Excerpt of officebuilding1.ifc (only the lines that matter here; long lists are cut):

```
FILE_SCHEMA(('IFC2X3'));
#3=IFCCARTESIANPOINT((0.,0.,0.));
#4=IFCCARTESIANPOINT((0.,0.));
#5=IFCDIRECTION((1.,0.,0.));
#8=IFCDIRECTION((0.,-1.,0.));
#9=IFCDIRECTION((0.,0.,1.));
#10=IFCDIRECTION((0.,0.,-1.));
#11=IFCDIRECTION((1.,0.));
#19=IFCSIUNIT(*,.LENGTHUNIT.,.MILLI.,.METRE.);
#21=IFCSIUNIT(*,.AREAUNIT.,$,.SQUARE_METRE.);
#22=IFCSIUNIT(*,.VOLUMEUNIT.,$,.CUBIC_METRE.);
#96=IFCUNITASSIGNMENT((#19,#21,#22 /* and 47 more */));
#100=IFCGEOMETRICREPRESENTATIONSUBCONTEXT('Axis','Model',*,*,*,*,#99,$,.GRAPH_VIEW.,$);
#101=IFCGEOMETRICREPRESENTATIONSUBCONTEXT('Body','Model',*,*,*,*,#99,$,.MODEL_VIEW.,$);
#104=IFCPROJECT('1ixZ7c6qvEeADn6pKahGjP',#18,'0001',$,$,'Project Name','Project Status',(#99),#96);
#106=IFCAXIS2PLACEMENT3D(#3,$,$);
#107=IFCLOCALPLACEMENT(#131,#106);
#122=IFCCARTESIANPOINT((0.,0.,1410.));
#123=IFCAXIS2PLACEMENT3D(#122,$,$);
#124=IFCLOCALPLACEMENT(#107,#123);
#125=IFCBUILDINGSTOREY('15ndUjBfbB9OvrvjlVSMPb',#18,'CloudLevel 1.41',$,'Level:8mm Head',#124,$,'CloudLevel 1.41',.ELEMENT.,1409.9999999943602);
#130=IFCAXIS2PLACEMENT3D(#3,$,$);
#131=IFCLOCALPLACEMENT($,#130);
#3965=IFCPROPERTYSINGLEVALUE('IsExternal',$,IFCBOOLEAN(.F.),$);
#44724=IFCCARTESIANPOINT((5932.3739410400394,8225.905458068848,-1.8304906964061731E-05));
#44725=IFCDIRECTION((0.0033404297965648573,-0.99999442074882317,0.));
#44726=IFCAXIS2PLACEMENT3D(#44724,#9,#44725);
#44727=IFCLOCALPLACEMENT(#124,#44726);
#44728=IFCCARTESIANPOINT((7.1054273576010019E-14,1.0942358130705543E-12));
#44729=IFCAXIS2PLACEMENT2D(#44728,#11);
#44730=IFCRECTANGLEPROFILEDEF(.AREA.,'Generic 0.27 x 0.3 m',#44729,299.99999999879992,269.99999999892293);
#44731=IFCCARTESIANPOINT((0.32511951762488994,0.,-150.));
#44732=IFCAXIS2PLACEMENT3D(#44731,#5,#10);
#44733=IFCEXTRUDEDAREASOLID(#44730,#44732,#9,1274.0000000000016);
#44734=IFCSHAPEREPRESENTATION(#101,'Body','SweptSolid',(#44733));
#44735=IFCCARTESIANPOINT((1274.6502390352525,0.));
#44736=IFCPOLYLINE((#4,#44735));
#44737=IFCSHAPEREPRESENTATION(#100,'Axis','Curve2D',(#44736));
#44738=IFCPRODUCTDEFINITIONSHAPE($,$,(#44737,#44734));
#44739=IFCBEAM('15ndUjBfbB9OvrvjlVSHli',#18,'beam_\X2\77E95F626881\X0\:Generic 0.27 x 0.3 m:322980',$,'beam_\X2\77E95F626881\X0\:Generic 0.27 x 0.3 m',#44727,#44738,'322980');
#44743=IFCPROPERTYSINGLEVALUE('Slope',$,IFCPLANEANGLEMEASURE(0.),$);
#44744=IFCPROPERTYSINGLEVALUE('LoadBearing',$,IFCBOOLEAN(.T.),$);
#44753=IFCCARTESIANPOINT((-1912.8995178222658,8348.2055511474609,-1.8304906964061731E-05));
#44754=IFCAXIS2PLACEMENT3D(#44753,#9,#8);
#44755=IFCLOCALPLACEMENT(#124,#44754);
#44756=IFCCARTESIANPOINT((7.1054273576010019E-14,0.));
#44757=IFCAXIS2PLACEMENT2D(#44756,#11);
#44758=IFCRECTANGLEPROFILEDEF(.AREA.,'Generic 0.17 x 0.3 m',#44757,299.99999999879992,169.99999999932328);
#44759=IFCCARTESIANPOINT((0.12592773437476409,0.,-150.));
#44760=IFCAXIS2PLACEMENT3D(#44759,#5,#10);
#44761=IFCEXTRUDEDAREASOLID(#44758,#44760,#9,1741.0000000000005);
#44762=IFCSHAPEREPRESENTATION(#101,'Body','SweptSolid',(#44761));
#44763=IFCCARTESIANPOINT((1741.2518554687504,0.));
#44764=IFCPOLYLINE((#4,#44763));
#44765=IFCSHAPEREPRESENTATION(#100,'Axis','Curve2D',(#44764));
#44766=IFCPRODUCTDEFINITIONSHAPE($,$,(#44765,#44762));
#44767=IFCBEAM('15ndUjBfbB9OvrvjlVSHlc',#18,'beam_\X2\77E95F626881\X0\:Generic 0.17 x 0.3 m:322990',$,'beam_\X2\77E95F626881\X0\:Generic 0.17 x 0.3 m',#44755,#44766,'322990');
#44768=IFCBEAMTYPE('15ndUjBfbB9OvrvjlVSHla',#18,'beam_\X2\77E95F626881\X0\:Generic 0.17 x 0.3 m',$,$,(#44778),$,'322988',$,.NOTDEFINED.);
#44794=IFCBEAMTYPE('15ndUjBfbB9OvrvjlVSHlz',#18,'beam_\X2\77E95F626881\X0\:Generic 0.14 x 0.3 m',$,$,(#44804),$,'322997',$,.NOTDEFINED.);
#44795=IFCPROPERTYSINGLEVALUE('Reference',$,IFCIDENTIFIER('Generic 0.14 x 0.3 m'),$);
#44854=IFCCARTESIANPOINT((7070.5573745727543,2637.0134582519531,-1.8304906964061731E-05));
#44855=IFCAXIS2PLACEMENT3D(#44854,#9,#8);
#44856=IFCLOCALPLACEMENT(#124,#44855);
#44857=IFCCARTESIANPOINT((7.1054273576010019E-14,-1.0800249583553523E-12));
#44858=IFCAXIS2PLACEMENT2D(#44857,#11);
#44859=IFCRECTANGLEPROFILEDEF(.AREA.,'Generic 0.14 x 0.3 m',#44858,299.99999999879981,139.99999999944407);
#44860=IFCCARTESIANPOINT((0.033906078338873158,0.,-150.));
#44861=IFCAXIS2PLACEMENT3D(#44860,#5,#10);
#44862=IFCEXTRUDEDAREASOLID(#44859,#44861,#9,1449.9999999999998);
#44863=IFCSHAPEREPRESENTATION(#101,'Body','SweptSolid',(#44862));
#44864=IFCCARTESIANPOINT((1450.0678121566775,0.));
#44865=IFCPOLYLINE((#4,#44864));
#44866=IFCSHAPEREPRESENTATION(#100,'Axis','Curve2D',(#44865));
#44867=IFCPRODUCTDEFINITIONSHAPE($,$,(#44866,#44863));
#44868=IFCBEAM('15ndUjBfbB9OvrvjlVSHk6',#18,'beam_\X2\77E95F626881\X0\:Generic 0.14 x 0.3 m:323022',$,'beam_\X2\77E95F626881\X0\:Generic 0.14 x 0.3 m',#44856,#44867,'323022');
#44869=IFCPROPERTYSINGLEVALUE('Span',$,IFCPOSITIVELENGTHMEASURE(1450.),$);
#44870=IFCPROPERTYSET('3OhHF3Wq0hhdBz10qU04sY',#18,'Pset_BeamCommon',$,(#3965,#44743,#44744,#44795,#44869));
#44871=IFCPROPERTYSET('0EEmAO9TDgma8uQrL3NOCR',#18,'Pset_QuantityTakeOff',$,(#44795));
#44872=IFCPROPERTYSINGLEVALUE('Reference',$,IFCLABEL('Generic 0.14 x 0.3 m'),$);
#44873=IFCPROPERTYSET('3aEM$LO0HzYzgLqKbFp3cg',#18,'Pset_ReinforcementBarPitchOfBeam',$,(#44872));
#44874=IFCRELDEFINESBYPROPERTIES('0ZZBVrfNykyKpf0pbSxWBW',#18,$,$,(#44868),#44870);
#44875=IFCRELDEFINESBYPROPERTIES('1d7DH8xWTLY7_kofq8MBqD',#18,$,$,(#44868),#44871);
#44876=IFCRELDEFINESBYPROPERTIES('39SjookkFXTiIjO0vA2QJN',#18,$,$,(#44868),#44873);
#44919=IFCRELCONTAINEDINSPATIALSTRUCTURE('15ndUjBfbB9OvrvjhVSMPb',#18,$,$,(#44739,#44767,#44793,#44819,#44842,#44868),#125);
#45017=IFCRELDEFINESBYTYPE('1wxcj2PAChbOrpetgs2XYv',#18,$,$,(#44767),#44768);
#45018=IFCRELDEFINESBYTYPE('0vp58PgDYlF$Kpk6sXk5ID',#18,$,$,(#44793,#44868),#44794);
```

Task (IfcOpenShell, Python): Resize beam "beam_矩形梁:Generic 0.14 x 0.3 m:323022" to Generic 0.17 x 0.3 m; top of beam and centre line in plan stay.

```python
import ifcopenshell
import ifcopenshell.api.pset
import ifcopenshell.api.type
import ifcopenshell.util.element
import ifcopenshell.util.representation

model = ifcopenshell.open("officebuilding1.ifc")

member = model.by_guid("15ndUjBfbB9OvrvjlVSHk6")
source = next(p for p in model.by_type("IfcRectangleProfileDef") if p.ProfileName == "Generic 0.17 x 0.3 m")

body = ifcopenshell.util.representation.get_representation(member, "Model", "Body")
solid = body.Items[0]
old_profile = solid.SweptArea

# Copy the section's sizes but keep this member's own profile position.
profile = ifcopenshell.util.element.copy(model, source)
# Profiles are centred, so shift by half the change in depth to hold the top.
shift = (old_profile.XDim - profile.XDim) / 2
x, y = old_profile.Position.Location.Coordinates
up = (-1.0, 0.0)  # upwards, in the solid's own plane
location = model.createIfcCartesianPoint((x + up[0] * shift, y + up[1] * shift))
profile.Position = model.createIfcAxis2Placement2D(location, old_profile.Position.RefDirection)
solid.SweptArea = profile
if not model.get_total_inverses(old_profile):
    ifcopenshell.util.element.remove_deep2(model, old_profile)

new_type = model.by_guid("15ndUjBfbB9OvrvjlVSHla")
ifcopenshell.api.type.assign_type(
    model, related_objects=[member], relating_type=new_type, should_map_representations=False
)
member.Name = member.Name.replace("Generic 0.14 x 0.3 m", "Generic 0.17 x 0.3 m")
member.ObjectType = "beam_矩形梁:Generic 0.17 x 0.3 m"
pset = model.by_id(ifcopenshell.util.element.get_pset(member, "Pset_BeamCommon", should_inherit=False)["id"])
ifcopenshell.api.pset.edit_pset(model, pset=pset, properties={"Reference": "Generic 0.17 x 0.3 m"})
pset = model.by_id(ifcopenshell.util.element.get_pset(member, "Pset_QuantityTakeOff", should_inherit=False)["id"])
ifcopenshell.api.pset.edit_pset(model, pset=pset, properties={"Reference": "Generic 0.17 x 0.3 m"})
pset = model.by_id(ifcopenshell.util.element.get_pset(member, "Pset_ReinforcementBarPitchOfBeam", should_inherit=False)["id"])
ifcopenshell.api.pset.edit_pset(model, pset=pset, properties={"Reference": "Generic 0.17 x 0.3 m"})

print(solid.SweptArea)

model.write("officebuilding1_v2.ifc")
```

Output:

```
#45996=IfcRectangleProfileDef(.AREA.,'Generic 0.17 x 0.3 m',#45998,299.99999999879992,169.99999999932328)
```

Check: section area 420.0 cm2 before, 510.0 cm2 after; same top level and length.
